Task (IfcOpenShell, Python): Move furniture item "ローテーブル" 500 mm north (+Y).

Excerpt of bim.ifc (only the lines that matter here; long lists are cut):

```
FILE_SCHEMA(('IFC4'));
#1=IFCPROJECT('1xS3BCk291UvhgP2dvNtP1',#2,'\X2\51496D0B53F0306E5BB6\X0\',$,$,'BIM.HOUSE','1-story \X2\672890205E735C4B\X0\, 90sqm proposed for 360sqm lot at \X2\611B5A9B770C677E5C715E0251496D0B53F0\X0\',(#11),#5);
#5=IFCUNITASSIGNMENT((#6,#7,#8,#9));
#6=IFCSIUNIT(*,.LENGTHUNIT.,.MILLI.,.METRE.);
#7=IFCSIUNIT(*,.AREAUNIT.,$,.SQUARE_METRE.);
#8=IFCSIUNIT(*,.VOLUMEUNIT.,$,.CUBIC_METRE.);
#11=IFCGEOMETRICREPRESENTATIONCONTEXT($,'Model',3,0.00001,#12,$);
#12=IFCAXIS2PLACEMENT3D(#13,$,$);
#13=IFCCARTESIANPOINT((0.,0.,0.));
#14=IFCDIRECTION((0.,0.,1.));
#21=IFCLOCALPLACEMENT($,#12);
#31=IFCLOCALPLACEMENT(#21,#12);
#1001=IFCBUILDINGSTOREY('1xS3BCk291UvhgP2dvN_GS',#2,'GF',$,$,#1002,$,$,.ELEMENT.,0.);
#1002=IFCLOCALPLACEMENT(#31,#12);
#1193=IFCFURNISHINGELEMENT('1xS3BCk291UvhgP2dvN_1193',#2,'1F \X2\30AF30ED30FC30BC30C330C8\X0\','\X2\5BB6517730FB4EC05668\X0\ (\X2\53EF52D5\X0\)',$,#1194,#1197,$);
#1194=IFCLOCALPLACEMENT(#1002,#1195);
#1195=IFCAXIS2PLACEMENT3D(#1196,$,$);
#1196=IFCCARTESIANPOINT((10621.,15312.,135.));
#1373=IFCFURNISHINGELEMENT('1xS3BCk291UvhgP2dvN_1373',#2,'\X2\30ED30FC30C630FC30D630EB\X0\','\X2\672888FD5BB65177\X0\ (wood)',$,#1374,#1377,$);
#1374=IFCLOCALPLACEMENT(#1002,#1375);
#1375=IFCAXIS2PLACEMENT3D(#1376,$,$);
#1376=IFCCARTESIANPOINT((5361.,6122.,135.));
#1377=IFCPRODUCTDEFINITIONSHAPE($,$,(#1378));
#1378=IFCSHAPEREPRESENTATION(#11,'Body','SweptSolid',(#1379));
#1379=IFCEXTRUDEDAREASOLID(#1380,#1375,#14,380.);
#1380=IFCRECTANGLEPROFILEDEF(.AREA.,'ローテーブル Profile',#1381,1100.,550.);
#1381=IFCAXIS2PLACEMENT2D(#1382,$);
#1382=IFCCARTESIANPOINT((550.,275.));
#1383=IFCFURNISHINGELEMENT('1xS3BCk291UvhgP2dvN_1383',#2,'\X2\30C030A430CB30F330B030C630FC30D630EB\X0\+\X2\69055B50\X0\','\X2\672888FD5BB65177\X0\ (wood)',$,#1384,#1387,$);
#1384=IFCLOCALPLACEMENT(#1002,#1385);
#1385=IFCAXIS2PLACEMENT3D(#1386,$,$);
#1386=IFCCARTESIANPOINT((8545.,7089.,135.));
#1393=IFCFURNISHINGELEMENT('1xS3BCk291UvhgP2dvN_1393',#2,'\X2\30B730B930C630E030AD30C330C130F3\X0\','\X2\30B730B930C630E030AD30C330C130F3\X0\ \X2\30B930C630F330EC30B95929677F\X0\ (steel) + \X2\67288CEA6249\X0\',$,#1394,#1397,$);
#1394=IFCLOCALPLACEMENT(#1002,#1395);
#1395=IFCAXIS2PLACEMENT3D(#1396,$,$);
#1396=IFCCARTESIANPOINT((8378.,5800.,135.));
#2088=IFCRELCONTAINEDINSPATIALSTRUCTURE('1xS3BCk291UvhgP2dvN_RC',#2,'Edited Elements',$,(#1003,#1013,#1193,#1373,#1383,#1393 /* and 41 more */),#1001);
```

```python
import ifcopenshell
import ifcopenshell.api.geometry
import ifcopenshell.util.placement
import ifcopenshell.util.unit

model = ifcopenshell.open("bim.ifc")
unit_scale = ifcopenshell.util.unit.calculate_unit_scale(model)

item = model.by_guid("1xS3BCk291UvhgP2dvN_1373")
matrix = ifcopenshell.util.placement.get_local_placement(item.ObjectPlacement)
matrix[1, 3] += 0.5 / unit_scale
ifcopenshell.api.geometry.edit_object_placement(model, product=item, matrix=matrix, is_si=False)

print(ifcopenshell.util.placement.get_local_placement(item.ObjectPlacement).round(3) + 0.0)

model.write("bim_edited.ifc")
```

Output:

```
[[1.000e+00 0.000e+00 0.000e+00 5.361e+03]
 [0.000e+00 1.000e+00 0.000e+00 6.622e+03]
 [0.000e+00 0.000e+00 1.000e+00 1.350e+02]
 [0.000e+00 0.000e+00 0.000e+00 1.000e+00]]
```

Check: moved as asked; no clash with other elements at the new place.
